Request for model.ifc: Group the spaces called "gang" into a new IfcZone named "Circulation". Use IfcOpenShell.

First a look at what the model holds.

```python
import ifcopenshell

model = ifcopenshell.open("model.ifc")
print(model.schema)
seen = {}
for space in model.by_type("IfcSpace"):
    seen[space.LongName] = seen.get(space.LongName, 0) + 1
for name, count in sorted(seen.items(), key=str):
    print(count, "x", name)
print("zones:", [z.Name for z in model.by_type("IfcZone")][:20])
```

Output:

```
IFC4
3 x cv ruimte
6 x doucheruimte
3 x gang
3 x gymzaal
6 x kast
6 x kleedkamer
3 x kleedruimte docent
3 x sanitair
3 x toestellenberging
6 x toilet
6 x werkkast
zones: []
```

```python
import ifcopenshell
import ifcopenshell.api.group
import ifcopenshell.api.root

model = ifcopenshell.open("model.ifc")

names = {"gang"}
spaces = [s for s in model.by_type("IfcSpace") if s.LongName in names]

zone = ifcopenshell.api.root.create_entity(model, ifc_class="IfcZone", name="Circulation")
ifcopenshell.api.group.assign_group(model, products=spaces, group=zone)
print(len(spaces), "spaces in", zone.Name)

model.write("model_v2.ifc")
```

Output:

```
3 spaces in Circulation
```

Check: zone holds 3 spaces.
